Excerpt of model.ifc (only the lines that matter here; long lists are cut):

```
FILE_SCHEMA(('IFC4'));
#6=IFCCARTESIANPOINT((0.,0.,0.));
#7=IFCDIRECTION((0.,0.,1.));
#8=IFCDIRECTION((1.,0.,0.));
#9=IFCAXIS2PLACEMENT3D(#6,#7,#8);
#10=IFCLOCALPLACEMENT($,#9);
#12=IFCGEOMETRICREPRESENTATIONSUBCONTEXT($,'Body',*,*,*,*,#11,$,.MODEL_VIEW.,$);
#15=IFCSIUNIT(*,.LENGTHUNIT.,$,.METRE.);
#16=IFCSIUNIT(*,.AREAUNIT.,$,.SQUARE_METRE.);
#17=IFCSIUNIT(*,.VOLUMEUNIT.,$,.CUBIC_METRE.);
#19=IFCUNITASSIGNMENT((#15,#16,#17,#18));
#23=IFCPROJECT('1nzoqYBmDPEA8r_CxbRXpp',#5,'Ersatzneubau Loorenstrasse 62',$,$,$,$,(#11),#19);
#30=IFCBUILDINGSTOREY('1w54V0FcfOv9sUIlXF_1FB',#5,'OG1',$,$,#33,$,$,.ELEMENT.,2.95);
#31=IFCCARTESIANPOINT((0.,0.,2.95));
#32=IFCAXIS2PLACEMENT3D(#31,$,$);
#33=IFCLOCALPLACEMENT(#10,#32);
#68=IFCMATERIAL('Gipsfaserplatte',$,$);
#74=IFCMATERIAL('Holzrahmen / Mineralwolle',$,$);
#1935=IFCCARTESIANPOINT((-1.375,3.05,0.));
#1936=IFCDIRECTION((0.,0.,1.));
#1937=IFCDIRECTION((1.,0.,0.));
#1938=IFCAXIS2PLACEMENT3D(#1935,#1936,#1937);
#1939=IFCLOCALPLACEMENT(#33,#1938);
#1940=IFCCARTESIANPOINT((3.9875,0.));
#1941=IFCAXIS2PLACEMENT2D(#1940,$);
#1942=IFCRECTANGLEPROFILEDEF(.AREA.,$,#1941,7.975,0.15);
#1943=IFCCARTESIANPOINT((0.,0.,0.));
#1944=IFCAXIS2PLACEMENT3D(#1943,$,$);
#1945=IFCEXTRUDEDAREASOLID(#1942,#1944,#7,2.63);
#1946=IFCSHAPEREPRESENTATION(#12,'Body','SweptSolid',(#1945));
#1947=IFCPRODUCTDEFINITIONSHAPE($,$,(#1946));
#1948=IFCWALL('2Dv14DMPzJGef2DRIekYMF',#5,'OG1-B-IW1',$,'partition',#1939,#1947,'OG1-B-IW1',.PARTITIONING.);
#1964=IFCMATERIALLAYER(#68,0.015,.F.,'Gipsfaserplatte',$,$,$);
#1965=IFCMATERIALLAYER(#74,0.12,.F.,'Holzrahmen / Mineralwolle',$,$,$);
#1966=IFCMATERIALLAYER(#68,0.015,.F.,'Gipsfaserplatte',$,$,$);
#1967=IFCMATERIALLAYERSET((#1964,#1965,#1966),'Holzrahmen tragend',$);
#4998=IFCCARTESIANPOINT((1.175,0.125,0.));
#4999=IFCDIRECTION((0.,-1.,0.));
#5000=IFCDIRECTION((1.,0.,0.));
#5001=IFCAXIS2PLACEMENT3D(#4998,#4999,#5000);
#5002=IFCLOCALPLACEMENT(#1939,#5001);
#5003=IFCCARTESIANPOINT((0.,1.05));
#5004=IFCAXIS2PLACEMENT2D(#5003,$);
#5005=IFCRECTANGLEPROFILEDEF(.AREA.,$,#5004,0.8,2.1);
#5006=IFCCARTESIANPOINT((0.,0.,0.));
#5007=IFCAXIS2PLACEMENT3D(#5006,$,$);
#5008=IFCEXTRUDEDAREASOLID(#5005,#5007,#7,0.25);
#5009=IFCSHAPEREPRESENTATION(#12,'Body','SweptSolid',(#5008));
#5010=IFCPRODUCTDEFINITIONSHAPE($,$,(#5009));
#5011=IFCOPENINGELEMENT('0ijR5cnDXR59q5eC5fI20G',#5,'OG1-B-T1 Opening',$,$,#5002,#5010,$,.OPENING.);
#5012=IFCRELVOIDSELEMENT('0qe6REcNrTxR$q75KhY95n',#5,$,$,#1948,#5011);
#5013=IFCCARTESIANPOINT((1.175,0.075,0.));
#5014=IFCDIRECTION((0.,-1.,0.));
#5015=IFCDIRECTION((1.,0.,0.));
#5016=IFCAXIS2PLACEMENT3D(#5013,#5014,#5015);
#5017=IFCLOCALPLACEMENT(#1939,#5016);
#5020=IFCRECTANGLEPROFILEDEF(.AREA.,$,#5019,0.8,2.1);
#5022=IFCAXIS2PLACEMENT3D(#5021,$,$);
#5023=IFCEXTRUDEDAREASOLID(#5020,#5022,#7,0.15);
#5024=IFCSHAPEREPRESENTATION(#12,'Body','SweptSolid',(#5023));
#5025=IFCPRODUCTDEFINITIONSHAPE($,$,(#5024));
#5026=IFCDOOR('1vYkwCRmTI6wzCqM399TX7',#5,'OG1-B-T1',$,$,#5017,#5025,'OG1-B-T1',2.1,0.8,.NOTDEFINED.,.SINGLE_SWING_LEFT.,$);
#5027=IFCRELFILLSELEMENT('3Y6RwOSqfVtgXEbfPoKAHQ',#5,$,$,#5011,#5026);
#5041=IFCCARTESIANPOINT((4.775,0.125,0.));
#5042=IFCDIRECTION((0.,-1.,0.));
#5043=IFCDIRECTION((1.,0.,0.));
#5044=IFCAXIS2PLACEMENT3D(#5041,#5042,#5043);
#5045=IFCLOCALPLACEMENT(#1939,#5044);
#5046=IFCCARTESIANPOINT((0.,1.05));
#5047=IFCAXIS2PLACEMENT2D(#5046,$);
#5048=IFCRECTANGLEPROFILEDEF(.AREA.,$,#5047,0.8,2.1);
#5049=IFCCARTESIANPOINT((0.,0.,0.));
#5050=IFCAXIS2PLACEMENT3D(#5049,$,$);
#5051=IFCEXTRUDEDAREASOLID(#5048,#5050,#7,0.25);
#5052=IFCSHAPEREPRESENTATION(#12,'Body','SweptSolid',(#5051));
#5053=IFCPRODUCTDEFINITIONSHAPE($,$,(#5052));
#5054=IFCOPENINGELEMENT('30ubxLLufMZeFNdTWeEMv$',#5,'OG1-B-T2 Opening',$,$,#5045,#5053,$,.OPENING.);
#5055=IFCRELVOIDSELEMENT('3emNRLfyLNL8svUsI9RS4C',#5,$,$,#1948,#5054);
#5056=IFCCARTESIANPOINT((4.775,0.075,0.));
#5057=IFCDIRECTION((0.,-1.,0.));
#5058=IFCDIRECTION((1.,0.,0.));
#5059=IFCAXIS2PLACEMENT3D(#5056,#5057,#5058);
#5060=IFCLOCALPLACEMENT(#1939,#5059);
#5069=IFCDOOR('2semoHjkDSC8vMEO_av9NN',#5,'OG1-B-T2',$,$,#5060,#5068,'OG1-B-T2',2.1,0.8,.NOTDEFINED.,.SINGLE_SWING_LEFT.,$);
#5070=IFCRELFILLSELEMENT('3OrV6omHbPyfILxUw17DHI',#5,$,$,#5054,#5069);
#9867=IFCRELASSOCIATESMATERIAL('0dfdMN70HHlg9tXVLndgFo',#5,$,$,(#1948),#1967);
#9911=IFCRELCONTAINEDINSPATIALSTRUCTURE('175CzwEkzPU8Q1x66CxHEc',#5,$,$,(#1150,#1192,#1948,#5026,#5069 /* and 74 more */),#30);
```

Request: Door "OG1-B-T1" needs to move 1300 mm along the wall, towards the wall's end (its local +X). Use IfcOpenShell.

```python
import ifcopenshell
import ifcopenshell.api.geometry
import ifcopenshell.util.placement
import ifcopenshell.util.unit

model = ifcopenshell.open("model.ifc")
unit_scale = ifcopenshell.util.unit.calculate_unit_scale(model)

door = model.by_id(5026)
opening = door.FillsVoids[0].RelatingOpeningElement
wall = opening.VoidsElements[0].RelatingBuildingElement

wall_matrix = ifcopenshell.util.placement.get_local_placement(wall.ObjectPlacement)
shift = wall_matrix[:3, 0] * 1.3 / unit_scale
before = ifcopenshell.util.placement.get_local_placement(door.ObjectPlacement)[:3, 3].copy()

# The door is not placed relative to its opening, so move both.
for product in (opening, door):
    matrix = ifcopenshell.util.placement.get_local_placement(product.ObjectPlacement)
    matrix[:3, 3] += shift
    ifcopenshell.api.geometry.edit_object_placement(model, product=product, matrix=matrix, is_si=False)

after = ifcopenshell.util.placement.get_local_placement(door.ObjectPlacement)[:3, 3]
print("door moved by", (after - before).round(3) + 0.0)

model.write("model_rev.ifc")
```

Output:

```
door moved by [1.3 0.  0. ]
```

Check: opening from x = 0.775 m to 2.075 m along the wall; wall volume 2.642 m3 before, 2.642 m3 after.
